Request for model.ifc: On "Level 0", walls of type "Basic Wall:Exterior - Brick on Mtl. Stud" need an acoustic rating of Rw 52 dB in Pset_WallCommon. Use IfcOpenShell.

First a look at what the model holds.

```python
import ifcopenshell
import ifcopenshell.util.element

model = ifcopenshell.open("model.ifc")
print(model.schema)
storey = next(s for s in model.by_type("IfcBuildingStorey") if s.Name == "Level 0")
walls = [e for e in ifcopenshell.util.element.get_decomposition(storey) if e.is_a("IfcWall")]
seen = {}
for e in walls:
    element_type = ifcopenshell.util.element.get_type(e)
    key = (element_type.Name if element_type != e and element_type else None, ifcopenshell.util.element.get_pset(e, "Pset_WallCommon", "AcousticRating"))
    seen[key] = seen.get(key, 0) + 1
for (name, value), count in sorted(seen.items(), key=str):
    print(count, "x", name, "|", value)
```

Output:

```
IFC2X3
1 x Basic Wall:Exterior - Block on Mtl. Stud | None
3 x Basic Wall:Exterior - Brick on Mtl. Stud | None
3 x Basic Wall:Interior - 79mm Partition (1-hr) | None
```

```python
import ifcopenshell
import ifcopenshell.api.pset
import ifcopenshell.util.element

model = ifcopenshell.open("model.ifc")

storey = next(s for s in model.by_type("IfcBuildingStorey") if s.Name == "Level 0")
walls = [e for e in ifcopenshell.util.element.get_decomposition(storey) if e.is_a("IfcWall")]

count = 0
for e in walls:
    element_type = ifcopenshell.util.element.get_type(e)
    if element_type in (None, e) or element_type.Name != "Basic Wall:Exterior - Brick on Mtl. Stud":
        continue
    # add_pset returns the element's existing set when there is one.
    pset = ifcopenshell.api.pset.add_pset(model, product=e, name="Pset_WallCommon")
    ifcopenshell.api.pset.edit_pset(model, pset=pset, properties={"AcousticRating": "Rw 52 dB"})
    count += 1

print(count, "walls updated")

model.write("model_rev.ifc")
```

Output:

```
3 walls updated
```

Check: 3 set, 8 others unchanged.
